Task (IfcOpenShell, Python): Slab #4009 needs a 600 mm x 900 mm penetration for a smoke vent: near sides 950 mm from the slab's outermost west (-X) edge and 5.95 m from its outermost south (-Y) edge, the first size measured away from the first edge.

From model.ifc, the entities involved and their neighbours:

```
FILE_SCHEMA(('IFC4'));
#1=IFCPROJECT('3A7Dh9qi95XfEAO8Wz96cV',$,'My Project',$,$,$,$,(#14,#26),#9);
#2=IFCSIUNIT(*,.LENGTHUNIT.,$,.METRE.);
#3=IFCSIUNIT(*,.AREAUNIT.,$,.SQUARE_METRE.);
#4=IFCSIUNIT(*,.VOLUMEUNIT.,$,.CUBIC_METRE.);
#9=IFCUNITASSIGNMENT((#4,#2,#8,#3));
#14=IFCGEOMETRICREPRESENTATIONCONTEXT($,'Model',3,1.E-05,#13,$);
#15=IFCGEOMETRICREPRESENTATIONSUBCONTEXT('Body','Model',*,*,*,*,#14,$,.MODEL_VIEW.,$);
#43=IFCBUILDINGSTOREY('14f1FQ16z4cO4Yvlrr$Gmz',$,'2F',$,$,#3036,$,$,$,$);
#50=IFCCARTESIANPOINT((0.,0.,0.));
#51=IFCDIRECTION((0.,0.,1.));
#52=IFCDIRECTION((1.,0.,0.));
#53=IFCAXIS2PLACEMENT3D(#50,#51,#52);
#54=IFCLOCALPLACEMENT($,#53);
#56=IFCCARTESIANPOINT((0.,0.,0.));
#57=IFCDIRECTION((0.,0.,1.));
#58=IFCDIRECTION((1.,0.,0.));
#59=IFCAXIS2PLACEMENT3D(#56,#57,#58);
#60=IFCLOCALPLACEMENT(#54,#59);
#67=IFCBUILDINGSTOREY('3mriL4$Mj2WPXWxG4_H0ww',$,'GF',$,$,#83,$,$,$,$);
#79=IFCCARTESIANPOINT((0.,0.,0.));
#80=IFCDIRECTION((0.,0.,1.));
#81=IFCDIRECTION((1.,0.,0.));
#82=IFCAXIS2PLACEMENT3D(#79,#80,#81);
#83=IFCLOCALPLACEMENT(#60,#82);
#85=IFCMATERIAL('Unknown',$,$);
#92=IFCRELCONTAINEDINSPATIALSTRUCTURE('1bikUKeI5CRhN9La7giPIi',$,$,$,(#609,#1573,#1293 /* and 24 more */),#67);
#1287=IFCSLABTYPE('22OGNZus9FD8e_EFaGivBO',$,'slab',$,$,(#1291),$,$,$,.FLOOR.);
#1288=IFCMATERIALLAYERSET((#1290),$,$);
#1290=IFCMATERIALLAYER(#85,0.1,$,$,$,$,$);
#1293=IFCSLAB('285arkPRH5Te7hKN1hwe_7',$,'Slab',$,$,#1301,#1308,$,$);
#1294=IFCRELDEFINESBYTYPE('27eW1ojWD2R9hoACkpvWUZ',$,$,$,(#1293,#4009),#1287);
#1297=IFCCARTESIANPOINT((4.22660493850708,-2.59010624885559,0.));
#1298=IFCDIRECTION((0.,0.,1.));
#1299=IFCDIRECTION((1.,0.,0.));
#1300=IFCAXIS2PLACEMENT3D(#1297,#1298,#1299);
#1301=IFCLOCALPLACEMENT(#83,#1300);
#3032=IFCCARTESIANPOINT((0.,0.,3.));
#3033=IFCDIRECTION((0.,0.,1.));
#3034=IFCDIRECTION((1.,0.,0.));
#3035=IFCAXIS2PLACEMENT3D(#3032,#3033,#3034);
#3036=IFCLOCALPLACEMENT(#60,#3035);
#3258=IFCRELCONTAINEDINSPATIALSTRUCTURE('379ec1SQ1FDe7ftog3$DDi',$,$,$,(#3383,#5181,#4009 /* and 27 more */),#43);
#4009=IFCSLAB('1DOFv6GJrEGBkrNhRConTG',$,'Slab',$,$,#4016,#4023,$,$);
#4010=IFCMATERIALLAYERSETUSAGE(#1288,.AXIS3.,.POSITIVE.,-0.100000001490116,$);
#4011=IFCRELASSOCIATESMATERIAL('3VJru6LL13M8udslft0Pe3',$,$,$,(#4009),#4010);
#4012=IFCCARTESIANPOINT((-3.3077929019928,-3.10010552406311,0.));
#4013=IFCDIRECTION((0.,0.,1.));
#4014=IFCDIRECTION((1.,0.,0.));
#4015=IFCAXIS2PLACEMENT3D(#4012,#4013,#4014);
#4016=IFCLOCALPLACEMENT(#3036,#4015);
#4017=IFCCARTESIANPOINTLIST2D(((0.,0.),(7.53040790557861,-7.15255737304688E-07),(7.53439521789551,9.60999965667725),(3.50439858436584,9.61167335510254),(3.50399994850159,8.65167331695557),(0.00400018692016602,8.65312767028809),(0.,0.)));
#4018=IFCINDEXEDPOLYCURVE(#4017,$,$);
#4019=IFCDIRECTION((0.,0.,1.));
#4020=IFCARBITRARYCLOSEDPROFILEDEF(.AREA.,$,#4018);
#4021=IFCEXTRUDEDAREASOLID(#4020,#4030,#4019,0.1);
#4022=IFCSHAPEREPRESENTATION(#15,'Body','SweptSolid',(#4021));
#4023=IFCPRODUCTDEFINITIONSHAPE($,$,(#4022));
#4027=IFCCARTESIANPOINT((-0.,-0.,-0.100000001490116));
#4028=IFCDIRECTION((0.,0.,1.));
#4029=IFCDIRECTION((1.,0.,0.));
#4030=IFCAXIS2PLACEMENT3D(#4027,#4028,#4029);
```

```python
import numpy as np
import ifcopenshell
import ifcopenshell.api.feature
import ifcopenshell.api.geometry
import ifcopenshell.api.root
import ifcopenshell.geom
import ifcopenshell.util.placement
import ifcopenshell.util.representation
import ifcopenshell.util.shape
import ifcopenshell.util.unit

model = ifcopenshell.open("model.ifc")
unit_scale = ifcopenshell.util.unit.calculate_unit_scale(model)
settings = ifcopenshell.geom.settings()


def volume(element):
    """Net volume in cubic metres, openings subtracted."""
    shape = ifcopenshell.geom.create_shape(settings, element)
    return ifcopenshell.util.shape.get_volume(shape.geometry)


slab = model.by_guid("1DOFv6GJrEGBkrNhRConTG")
before = volume(slab)

# Extent in the slab's own axes, in metres. The edges named are its -X and -Y sides.
slab_shape = ifcopenshell.geom.create_shape(settings, slab)
vertices = ifcopenshell.util.shape.get_vertices(slab_shape.geometry)
x_min, y_min, bottom = vertices.min(axis=0)
top = vertices[:, 2].max()

opening = ifcopenshell.api.root.create_entity(model, ifc_class="IfcOpeningElement", name="Smoke vent opening", predefined_type="OPENING")
context = ifcopenshell.util.representation.get_context(model, "Model", "Body", "MODEL_VIEW")
width, depth = 0.6, 0.9
outline = [(0.0, 0.0), (width, 0.0), (width, depth), (0.0, depth), (0.0, 0.0)]
# Overshoot both faces by 50 mm so the cut is clean.
shape = ifcopenshell.api.geometry.add_slab_representation(
    model, context=context, depth=top - bottom + 0.1, polyline=outline
)
ifcopenshell.api.geometry.assign_representation(model, product=opening, representation=shape)

matrix = ifcopenshell.util.placement.get_local_placement(slab.ObjectPlacement)
matrix[:, 3] = matrix @ np.append(np.array([x_min + 0.95, y_min + 5.95, bottom - 0.05]) / unit_scale, 1.0)
ifcopenshell.api.geometry.edit_object_placement(model, product=opening, matrix=matrix, is_si=False)
ifcopenshell.api.feature.add_feature(model, feature=opening, element=slab)

after = volume(slab)

print(f"slab volume {before:.3f} -> {after:.3f} m3")

model.write("model_rev.ifc")
```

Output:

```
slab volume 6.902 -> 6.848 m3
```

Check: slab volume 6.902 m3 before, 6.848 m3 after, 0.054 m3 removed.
